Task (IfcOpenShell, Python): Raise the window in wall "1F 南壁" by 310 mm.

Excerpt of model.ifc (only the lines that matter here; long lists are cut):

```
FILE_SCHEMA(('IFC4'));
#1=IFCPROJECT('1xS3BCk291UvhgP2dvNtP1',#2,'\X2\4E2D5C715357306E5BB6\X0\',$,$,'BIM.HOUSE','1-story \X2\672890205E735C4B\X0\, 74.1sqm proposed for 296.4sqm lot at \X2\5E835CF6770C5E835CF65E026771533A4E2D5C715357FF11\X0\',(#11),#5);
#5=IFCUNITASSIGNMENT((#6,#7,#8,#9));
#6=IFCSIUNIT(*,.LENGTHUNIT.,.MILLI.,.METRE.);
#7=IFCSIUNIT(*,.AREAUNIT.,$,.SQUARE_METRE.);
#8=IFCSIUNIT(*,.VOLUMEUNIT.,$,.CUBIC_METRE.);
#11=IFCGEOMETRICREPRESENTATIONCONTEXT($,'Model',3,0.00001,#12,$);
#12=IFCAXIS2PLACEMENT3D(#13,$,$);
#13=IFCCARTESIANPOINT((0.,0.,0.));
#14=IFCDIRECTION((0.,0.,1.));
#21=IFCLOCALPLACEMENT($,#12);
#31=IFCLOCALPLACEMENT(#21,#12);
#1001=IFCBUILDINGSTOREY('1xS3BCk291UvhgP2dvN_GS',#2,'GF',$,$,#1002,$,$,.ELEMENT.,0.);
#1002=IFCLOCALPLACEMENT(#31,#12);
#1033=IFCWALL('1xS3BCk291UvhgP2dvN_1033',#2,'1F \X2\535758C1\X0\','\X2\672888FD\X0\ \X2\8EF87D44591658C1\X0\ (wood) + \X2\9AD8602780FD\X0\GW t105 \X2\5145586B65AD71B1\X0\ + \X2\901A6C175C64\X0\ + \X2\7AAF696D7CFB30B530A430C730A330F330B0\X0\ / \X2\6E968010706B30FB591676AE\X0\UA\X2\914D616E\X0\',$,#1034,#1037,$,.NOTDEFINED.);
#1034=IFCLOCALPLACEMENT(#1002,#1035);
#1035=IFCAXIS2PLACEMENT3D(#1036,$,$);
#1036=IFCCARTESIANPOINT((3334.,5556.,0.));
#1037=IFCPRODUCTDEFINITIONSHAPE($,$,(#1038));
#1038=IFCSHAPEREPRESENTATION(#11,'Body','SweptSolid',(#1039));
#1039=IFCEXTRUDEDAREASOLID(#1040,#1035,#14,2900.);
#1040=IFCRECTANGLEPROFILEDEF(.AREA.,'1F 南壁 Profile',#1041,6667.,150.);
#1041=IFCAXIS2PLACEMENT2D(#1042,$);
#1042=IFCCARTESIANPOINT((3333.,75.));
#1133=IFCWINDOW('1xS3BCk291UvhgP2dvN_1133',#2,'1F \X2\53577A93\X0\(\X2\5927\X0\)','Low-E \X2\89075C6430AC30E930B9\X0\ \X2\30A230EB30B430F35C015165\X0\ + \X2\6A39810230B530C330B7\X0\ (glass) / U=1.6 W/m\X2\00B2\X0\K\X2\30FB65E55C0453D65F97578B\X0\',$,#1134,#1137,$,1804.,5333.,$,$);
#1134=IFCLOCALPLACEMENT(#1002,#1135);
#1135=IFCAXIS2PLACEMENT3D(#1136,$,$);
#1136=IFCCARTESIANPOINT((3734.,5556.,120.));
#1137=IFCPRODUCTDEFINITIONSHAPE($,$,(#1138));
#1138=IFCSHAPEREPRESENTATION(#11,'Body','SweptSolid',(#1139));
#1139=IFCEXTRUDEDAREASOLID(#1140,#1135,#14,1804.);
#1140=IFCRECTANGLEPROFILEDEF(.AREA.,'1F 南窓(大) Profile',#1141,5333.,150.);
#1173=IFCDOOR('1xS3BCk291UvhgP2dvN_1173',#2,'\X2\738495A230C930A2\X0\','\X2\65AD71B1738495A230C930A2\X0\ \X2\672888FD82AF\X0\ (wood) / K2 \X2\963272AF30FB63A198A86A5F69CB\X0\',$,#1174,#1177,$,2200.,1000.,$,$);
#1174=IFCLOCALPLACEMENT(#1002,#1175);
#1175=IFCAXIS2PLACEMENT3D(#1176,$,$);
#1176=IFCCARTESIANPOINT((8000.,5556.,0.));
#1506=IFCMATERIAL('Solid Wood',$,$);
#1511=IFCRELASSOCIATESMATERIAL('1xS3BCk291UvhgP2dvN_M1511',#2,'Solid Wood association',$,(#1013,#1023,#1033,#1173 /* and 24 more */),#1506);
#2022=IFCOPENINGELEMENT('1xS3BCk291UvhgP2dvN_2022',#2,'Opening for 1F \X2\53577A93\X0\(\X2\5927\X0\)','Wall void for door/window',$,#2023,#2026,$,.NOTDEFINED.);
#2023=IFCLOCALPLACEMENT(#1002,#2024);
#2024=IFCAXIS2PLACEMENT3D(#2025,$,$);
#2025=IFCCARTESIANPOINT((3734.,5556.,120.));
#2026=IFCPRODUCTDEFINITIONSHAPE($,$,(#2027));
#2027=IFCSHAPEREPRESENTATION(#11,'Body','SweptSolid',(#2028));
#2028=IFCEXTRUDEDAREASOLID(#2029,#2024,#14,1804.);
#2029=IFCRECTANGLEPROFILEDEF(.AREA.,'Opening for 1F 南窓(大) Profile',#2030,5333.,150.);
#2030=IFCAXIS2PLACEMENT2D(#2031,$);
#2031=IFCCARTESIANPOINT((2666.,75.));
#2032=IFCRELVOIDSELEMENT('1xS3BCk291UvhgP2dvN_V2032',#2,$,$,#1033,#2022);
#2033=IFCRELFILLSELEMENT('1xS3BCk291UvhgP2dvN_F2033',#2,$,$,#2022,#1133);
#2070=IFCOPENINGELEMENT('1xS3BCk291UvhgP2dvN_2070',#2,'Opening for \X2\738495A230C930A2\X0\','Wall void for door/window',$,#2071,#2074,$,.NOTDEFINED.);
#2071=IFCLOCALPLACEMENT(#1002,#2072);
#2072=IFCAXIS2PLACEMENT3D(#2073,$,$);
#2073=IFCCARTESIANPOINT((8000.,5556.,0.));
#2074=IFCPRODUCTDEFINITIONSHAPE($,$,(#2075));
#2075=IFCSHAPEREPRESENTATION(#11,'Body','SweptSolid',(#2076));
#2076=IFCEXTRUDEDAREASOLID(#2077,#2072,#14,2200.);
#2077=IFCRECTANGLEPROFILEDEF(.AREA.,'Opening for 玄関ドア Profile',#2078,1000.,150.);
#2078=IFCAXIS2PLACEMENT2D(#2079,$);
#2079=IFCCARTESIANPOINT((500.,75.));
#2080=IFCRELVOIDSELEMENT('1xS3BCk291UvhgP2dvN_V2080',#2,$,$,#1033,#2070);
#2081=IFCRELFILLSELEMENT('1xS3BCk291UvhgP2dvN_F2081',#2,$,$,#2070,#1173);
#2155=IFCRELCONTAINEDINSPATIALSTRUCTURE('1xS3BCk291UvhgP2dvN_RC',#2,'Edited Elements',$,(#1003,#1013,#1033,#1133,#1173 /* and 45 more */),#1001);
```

```python
import numpy as np
import ifcopenshell
import ifcopenshell.api.geometry
import ifcopenshell.util.placement
import ifcopenshell.util.unit

model = ifcopenshell.open("model.ifc")
unit_scale = ifcopenshell.util.unit.calculate_unit_scale(model)

window = model.by_guid("1xS3BCk291UvhgP2dvN_1133")
opening = window.FillsVoids[0].RelatingOpeningElement
dz = 0.31 / unit_scale

shift = np.array([0.0, 0.0, dz])
# The window is not placed relative to its opening, so move both.
for product in (opening, window):
    matrix = ifcopenshell.util.placement.get_local_placement(product.ObjectPlacement)
    matrix[:3, 3] += shift
    ifcopenshell.api.geometry.edit_object_placement(model, product=product, matrix=matrix, is_si=False)

print(f"moved by {dz * unit_scale:+.3f} m")

model.write("model_edited.ifc")
```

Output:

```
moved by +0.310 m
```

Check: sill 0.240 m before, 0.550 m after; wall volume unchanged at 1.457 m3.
